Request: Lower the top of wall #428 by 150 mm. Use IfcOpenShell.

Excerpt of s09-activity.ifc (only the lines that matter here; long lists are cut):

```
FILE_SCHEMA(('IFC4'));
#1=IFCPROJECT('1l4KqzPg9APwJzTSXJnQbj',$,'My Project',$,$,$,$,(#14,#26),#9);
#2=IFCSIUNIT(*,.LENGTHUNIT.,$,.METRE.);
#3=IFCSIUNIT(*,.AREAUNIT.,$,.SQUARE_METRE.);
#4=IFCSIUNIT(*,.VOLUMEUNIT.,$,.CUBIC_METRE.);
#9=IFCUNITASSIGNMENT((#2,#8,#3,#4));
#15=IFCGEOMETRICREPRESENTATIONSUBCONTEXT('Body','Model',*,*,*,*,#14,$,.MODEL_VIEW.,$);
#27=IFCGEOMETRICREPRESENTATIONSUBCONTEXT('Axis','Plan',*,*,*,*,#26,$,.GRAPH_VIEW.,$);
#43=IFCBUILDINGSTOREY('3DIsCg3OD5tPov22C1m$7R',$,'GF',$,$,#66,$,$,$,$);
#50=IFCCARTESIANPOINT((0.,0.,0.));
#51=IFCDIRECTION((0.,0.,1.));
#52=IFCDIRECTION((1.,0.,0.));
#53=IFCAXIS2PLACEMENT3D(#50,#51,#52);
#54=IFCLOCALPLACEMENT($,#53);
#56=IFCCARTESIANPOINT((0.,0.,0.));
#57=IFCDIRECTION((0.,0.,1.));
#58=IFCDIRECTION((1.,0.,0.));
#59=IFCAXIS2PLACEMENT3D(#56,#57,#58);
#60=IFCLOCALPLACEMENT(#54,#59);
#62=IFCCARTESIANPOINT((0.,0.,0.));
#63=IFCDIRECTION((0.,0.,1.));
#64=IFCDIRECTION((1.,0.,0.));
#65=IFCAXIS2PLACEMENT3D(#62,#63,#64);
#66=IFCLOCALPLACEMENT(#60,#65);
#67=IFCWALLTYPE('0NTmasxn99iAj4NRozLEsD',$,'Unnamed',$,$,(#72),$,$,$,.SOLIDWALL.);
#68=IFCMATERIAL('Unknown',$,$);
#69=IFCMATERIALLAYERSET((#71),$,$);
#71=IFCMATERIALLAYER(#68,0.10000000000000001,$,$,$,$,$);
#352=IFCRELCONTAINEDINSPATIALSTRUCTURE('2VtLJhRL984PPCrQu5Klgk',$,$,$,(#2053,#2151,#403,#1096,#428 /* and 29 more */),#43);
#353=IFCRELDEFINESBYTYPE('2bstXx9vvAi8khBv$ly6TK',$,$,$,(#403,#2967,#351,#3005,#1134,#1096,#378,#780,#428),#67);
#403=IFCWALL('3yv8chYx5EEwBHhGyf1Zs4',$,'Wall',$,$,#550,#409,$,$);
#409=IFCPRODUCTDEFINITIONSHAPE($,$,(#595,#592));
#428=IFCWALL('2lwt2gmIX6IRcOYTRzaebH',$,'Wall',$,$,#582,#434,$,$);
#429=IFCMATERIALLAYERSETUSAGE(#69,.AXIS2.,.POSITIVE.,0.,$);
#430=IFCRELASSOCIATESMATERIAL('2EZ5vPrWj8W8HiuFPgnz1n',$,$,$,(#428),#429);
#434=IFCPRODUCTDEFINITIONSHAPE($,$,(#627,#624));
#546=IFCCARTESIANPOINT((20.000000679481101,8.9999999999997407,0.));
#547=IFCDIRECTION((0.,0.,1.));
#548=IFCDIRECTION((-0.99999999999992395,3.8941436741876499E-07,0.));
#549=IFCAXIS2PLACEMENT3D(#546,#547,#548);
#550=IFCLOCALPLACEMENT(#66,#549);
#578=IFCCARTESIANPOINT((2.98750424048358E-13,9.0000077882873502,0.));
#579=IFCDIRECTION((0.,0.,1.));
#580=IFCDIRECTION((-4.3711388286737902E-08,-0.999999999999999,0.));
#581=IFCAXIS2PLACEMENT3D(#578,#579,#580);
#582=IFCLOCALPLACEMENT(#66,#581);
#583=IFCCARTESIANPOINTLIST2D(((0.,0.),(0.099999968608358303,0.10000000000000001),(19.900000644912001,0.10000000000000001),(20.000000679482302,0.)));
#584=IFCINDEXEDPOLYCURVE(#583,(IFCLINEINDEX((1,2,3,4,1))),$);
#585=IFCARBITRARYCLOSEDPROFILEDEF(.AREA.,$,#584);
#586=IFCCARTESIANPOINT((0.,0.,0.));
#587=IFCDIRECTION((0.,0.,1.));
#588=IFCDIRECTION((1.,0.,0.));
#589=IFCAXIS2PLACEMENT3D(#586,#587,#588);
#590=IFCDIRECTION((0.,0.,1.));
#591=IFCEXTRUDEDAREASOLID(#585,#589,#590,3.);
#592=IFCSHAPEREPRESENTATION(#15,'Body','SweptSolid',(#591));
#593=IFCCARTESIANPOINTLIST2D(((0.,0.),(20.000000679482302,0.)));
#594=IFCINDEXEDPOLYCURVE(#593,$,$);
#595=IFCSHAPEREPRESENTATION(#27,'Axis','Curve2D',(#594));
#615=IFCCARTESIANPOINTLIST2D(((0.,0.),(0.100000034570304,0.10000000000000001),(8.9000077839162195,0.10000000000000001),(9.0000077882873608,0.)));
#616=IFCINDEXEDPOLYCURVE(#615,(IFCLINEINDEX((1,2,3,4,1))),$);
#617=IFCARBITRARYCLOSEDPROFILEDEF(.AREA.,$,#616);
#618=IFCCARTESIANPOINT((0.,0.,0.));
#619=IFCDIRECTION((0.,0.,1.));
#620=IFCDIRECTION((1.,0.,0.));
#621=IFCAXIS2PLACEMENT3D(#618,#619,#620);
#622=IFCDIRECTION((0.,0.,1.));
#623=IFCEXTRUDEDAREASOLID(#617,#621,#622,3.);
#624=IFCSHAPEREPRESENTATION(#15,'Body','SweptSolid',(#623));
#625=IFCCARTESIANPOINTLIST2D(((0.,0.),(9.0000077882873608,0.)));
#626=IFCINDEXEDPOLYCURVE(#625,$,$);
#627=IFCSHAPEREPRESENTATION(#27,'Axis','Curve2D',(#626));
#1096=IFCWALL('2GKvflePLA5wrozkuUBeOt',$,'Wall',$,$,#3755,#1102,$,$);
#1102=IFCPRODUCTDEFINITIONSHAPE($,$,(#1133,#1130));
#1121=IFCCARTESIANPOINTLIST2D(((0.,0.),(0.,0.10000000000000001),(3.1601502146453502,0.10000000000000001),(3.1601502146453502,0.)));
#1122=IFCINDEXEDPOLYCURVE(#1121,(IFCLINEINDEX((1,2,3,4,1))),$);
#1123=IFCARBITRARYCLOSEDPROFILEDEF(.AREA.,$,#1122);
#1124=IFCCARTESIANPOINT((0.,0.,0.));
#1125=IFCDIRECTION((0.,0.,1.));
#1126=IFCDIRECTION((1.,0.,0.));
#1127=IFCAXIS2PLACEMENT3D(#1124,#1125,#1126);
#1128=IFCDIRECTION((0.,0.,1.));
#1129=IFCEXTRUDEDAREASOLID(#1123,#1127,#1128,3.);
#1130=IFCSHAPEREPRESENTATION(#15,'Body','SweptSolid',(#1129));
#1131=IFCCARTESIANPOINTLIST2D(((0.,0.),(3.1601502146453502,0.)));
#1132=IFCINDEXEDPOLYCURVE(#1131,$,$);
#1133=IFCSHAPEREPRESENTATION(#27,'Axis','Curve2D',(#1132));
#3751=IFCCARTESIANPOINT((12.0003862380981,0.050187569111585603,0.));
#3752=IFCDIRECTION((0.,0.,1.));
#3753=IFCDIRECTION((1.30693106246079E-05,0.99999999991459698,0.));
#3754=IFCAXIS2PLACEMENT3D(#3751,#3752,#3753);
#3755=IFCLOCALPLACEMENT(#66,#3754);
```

```python
import ifcopenshell
import ifcopenshell.geom
import ifcopenshell.util.representation
import ifcopenshell.util.shape
import ifcopenshell.util.unit

model = ifcopenshell.open("s09-activity.ifc")
unit_scale = ifcopenshell.util.unit.calculate_unit_scale(model)
settings = ifcopenshell.geom.settings()


def volume(element):
    """Net volume in cubic metres, openings subtracted."""
    shape = ifcopenshell.geom.create_shape(settings, element)
    return ifcopenshell.util.shape.get_volume(shape.geometry)


wall = model.by_id(428)
before = volume(wall)

body = ifcopenshell.util.representation.get_representation(wall, "Model", "Body")
solid = body.Items[0]
old_height = solid.Depth
solid.Depth -= 0.15 / unit_scale
after = volume(wall)

print(f"height {old_height:g} -> {solid.Depth:g}, volume {before:.3f} -> {after:.3f} m3")

model.write("s09-activity_updated.ifc")
```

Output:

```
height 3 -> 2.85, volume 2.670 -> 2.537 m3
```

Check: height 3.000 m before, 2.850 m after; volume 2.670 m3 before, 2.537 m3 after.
